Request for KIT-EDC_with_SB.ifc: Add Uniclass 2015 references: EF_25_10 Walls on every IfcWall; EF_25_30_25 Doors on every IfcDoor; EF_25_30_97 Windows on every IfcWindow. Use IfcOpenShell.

First a look at what the model holds.

```python
import ifcopenshell

model = ifcopenshell.open("KIT-EDC_with_SB.ifc")
print(model.schema)
print("classifications:", [c.Name for c in model.by_type("IfcClassification")])
for ifc_class in ("IfcDoor", "IfcRoof", "IfcStair", "IfcWall", "IfcWindow"):
    print(ifc_class, len(model.by_type(ifc_class)))
```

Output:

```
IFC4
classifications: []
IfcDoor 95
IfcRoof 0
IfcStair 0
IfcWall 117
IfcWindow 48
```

```python
import ifcopenshell
import ifcopenshell.api.classification

model = ifcopenshell.open("KIT-EDC_with_SB.ifc")

system = ifcopenshell.api.classification.add_classification(model, classification="Uniclass 2015")

codes = {
    "IfcWall": ("EF_25_10", "Walls"),
    "IfcDoor": ("EF_25_30_25", "Doors"),
    "IfcWindow": ("EF_25_30_97", "Windows"),
}
for ifc_class, (code, name) in codes.items():
    products = model.by_type(ifc_class)
    ifcopenshell.api.classification.add_reference(
        model, products=products, classification=system, identification=code, name=name
    )
    print(code, len(products))

model.write("KIT-EDC_with_SB_v2.ifc")
```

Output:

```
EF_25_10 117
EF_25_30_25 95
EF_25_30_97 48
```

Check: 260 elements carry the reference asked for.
